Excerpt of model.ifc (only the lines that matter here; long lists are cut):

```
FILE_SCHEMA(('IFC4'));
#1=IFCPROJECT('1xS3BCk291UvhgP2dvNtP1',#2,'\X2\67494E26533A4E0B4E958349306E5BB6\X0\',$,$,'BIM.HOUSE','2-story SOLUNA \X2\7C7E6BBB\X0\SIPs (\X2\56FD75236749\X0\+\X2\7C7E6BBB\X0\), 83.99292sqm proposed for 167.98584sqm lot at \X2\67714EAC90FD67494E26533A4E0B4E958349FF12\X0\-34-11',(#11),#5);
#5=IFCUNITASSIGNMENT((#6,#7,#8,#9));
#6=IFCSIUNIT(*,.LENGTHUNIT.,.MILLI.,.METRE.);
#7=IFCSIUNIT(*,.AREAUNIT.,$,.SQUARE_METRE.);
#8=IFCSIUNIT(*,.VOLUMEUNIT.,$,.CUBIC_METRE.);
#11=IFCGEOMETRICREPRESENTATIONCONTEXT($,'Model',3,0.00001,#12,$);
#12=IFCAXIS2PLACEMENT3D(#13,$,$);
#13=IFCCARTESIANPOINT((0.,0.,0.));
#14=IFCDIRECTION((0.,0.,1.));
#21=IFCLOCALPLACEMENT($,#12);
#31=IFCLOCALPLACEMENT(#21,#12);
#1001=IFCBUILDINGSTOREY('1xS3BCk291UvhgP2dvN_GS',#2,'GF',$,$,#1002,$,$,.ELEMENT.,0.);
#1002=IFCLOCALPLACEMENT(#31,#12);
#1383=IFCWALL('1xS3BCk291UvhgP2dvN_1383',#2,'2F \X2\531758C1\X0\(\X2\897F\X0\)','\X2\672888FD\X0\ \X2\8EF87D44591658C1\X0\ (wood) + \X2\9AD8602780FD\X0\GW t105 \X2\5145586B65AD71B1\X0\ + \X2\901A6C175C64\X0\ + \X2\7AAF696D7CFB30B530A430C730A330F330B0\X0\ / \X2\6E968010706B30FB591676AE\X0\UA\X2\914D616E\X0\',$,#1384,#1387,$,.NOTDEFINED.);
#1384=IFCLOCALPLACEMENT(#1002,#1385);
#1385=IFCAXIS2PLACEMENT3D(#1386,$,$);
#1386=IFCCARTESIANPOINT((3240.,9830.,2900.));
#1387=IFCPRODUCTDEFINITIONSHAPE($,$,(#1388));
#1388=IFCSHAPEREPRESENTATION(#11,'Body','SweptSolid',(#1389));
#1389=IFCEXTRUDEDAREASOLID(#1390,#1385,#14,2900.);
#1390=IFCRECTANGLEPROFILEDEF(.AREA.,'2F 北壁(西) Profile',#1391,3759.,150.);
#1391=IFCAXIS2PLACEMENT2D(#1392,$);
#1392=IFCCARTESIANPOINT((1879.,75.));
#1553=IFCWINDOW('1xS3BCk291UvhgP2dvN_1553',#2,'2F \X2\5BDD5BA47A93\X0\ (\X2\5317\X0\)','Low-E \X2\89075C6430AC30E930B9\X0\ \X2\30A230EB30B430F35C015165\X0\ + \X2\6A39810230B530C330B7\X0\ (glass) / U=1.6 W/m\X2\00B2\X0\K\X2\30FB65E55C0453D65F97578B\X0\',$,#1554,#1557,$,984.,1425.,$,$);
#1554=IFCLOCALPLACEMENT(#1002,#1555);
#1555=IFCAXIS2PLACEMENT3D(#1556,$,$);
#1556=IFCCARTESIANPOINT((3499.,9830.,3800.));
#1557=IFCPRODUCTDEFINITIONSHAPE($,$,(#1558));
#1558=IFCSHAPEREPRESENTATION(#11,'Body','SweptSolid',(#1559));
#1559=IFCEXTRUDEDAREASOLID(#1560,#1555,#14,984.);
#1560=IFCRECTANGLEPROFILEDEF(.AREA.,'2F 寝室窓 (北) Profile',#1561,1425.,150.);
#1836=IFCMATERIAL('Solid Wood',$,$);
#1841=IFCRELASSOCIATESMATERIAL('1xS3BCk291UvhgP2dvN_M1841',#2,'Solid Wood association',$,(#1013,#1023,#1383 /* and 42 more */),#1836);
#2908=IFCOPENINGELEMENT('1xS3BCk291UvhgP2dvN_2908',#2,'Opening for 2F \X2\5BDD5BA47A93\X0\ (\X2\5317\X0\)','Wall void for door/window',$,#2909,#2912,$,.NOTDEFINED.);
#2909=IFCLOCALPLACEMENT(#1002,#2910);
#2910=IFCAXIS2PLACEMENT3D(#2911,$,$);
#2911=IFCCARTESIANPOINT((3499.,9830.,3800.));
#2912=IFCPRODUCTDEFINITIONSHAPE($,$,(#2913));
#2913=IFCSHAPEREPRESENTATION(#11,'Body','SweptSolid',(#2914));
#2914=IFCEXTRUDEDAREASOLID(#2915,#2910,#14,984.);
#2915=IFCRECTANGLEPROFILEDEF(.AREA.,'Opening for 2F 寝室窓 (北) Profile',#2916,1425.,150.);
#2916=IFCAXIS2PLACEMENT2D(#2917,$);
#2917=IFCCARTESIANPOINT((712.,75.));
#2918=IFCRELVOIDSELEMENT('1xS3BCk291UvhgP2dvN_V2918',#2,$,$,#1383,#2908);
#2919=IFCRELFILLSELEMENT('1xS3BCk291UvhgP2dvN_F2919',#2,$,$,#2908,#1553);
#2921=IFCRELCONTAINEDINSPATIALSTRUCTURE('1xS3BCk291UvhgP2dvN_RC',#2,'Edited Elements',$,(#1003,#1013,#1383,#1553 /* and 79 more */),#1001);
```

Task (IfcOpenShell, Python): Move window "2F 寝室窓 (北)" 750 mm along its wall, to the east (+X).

```python
import ifcopenshell
import ifcopenshell.api.geometry
import ifcopenshell.util.placement
import ifcopenshell.util.unit

model = ifcopenshell.open("model.ifc")
unit_scale = ifcopenshell.util.unit.calculate_unit_scale(model)

window = model.by_id(1553)
opening = window.FillsVoids[0].RelatingOpeningElement
wall = opening.VoidsElements[0].RelatingBuildingElement

wall_matrix = ifcopenshell.util.placement.get_local_placement(wall.ObjectPlacement)
shift = wall_matrix[:3, 0] * 0.75 / unit_scale
before = ifcopenshell.util.placement.get_local_placement(window.ObjectPlacement)[:3, 3].copy()

# The window is not placed relative to its opening, so move both.
for product in (opening, window):
    matrix = ifcopenshell.util.placement.get_local_placement(product.ObjectPlacement)
    matrix[:3, 3] += shift
    ifcopenshell.api.geometry.edit_object_placement(model, product=product, matrix=matrix, is_si=False)

after = ifcopenshell.util.placement.get_local_placement(window.ObjectPlacement)[:3, 3]
print("window moved by", (after - before).round(3) + 0.0)

model.write("model_rev.ifc")
```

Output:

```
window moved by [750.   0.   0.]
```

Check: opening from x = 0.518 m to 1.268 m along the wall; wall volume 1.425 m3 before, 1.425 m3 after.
